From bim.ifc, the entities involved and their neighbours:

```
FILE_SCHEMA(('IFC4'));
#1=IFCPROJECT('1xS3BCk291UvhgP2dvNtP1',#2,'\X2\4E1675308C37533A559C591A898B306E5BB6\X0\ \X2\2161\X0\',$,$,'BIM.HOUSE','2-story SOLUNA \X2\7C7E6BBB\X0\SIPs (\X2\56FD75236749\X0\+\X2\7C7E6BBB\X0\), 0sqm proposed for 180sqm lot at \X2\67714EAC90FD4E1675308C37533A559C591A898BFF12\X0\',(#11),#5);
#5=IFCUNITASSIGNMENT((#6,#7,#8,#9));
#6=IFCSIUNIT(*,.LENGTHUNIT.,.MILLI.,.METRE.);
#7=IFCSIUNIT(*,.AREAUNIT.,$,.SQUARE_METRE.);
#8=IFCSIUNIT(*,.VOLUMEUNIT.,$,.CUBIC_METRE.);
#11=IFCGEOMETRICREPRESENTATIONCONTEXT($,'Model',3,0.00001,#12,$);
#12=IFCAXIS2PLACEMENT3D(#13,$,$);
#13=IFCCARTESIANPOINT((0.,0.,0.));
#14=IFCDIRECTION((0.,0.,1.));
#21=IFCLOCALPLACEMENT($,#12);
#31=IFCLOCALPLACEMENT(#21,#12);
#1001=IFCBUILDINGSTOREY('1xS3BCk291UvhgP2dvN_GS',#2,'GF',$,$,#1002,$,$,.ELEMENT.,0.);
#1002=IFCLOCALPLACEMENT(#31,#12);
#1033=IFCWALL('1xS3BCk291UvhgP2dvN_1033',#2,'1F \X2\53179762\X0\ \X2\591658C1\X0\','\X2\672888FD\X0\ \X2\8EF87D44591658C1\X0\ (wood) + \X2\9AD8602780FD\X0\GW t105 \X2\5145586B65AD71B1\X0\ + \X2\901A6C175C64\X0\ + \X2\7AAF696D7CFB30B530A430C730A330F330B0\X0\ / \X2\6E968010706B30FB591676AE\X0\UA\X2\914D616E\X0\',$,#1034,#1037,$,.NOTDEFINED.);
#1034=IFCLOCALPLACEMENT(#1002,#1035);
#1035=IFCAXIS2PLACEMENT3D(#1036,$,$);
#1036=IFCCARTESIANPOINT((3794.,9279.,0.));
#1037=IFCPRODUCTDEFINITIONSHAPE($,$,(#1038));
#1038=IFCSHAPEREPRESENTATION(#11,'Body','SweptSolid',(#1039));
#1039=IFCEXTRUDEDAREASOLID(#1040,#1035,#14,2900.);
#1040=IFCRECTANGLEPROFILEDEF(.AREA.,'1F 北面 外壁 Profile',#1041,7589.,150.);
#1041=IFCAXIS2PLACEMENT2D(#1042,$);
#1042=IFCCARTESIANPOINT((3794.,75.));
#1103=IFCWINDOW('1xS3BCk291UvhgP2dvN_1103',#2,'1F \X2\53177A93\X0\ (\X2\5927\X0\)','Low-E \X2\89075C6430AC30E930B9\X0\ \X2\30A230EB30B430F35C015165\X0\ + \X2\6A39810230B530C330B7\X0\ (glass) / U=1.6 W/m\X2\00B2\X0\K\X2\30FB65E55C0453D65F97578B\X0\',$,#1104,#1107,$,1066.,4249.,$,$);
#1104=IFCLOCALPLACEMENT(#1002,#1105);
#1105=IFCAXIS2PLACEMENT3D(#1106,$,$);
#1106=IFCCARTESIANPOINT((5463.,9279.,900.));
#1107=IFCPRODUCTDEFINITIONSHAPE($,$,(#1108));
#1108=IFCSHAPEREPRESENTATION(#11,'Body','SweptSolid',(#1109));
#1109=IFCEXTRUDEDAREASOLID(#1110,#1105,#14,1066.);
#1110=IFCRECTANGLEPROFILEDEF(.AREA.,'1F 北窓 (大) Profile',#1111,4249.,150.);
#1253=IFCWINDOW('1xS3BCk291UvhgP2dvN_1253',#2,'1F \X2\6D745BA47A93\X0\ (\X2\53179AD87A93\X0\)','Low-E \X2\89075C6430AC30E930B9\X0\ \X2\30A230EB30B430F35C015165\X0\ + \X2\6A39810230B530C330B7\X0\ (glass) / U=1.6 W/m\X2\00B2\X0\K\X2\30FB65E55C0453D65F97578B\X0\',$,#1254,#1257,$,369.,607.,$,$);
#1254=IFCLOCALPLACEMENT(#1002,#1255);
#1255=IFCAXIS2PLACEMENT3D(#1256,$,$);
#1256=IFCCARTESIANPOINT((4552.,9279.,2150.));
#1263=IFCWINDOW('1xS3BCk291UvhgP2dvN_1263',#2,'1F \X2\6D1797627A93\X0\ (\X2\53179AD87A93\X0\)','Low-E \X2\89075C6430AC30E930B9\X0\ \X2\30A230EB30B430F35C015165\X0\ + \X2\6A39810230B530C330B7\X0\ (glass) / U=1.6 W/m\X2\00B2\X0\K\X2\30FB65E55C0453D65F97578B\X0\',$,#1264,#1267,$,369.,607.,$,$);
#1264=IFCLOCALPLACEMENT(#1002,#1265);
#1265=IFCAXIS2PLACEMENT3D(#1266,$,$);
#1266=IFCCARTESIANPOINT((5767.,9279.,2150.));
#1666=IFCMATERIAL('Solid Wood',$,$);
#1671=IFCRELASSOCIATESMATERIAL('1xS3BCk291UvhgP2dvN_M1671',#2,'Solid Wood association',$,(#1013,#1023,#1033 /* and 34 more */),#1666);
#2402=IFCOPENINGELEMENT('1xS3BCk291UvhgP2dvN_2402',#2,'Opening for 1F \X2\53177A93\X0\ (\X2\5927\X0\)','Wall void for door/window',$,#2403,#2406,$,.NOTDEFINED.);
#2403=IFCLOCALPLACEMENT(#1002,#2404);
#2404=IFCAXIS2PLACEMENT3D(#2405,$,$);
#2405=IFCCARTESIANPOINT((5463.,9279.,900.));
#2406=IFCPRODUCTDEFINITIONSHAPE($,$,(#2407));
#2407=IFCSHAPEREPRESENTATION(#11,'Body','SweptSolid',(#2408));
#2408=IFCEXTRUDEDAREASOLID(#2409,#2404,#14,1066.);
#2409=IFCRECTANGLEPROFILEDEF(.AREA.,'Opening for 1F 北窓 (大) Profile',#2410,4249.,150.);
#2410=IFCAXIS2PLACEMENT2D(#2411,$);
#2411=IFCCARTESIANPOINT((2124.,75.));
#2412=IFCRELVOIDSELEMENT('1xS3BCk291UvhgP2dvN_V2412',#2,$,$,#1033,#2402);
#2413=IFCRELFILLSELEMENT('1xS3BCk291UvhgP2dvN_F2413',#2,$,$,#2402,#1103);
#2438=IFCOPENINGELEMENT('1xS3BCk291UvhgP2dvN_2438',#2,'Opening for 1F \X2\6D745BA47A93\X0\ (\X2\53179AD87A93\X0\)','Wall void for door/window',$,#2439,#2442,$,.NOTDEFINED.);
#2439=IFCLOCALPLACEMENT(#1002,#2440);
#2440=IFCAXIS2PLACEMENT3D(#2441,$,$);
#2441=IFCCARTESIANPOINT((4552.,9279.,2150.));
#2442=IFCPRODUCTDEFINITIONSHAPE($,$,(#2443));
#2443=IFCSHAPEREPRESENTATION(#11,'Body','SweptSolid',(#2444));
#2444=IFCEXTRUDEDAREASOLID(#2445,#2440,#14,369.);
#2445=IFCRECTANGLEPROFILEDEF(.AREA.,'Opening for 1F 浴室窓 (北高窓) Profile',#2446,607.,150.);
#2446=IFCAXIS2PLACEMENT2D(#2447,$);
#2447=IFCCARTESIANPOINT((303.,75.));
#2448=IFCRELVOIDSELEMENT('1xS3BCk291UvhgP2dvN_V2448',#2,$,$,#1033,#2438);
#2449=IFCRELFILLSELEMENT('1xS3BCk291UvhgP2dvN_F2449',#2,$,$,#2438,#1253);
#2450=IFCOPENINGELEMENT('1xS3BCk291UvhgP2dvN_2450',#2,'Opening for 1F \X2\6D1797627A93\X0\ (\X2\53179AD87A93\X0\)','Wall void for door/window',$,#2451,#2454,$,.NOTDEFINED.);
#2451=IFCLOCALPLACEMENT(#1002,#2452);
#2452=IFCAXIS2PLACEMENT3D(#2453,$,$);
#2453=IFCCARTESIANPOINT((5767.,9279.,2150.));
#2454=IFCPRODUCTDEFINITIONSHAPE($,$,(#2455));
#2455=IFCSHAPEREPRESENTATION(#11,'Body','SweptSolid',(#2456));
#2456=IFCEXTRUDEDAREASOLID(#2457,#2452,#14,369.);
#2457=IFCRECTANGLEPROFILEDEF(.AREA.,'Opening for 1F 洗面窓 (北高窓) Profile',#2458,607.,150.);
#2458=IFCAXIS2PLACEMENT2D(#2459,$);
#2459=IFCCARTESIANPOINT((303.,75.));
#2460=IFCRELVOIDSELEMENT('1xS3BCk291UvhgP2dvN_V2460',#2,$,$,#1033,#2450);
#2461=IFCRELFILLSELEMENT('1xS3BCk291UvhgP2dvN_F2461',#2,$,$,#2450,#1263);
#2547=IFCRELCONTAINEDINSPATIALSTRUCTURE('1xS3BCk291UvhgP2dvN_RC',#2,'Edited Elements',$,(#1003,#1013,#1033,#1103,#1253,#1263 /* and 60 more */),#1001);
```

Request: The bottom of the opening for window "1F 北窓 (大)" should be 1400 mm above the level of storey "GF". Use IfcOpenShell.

```python
import numpy as np
import ifcopenshell
import ifcopenshell.api.geometry
import ifcopenshell.geom
import ifcopenshell.util.element
import ifcopenshell.util.placement
import ifcopenshell.util.shape
import ifcopenshell.util.unit

model = ifcopenshell.open("bim.ifc")
unit_scale = ifcopenshell.util.unit.calculate_unit_scale(model)

window = model.by_guid("1xS3BCk291UvhgP2dvN_1103")
opening = window.FillsVoids[0].RelatingOpeningElement
storey = ifcopenshell.util.element.get_container(window, ifc_class="IfcBuildingStorey")
level = ifcopenshell.util.placement.get_local_placement(storey.ObjectPlacement)[2, 3]

# The opening's origin need not be at the sill, so measure its lowest point.
shape = ifcopenshell.geom.create_shape(ifcopenshell.geom.settings(), opening)
bottom = ifcopenshell.util.shape.get_shape_bottom_elevation(shape, shape.geometry) / unit_scale
dz = level + 1400.0 - bottom

shift = np.array([0.0, 0.0, dz])
# The window is not placed relative to its opening, so move both.
for product in (opening, window):
    matrix = ifcopenshell.util.placement.get_local_placement(product.ObjectPlacement)
    matrix[:3, 3] += shift
    ifcopenshell.api.geometry.edit_object_placement(model, product=product, matrix=matrix, is_si=False)

print(f"moved by {dz * unit_scale:+.3f} m")

model.write("bim_updated.ifc")
```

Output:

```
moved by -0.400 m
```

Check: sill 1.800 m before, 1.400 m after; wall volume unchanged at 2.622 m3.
